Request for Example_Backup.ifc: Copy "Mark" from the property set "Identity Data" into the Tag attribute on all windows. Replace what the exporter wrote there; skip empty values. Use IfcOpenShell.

First a look at what the model holds.

```python
import ifcopenshell
import ifcopenshell.util.element

model = ifcopenshell.open("Example_Backup.ifc")
print(model.schema)
windows = model.by_type("IfcWindow")
print(len(windows), "windows")
for e in windows[:8]:
    source = ifcopenshell.util.element.get_pset(e, "Identity Data", "Mark")
    target = e.Tag
    print(e.id(), repr(source), repr(target), sep=" | ")
```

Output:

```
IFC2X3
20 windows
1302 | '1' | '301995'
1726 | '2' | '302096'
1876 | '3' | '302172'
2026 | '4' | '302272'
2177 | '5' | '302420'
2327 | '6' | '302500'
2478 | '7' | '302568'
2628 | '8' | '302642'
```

```python
import ifcopenshell
import ifcopenshell.util.element

model = ifcopenshell.open("Example_Backup.ifc")

count = 0
for e in model.by_type("IfcWindow"):
    value = ifcopenshell.util.element.get_pset(e, "Identity Data", "Mark")
    current = e.Tag
    if not value or not value.strip() or current == value:
        continue
    e.Tag = value
    count += 1

print(count, "windows updated")

model.write("Example_Backup_updated.ifc")
```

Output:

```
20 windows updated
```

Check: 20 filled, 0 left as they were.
